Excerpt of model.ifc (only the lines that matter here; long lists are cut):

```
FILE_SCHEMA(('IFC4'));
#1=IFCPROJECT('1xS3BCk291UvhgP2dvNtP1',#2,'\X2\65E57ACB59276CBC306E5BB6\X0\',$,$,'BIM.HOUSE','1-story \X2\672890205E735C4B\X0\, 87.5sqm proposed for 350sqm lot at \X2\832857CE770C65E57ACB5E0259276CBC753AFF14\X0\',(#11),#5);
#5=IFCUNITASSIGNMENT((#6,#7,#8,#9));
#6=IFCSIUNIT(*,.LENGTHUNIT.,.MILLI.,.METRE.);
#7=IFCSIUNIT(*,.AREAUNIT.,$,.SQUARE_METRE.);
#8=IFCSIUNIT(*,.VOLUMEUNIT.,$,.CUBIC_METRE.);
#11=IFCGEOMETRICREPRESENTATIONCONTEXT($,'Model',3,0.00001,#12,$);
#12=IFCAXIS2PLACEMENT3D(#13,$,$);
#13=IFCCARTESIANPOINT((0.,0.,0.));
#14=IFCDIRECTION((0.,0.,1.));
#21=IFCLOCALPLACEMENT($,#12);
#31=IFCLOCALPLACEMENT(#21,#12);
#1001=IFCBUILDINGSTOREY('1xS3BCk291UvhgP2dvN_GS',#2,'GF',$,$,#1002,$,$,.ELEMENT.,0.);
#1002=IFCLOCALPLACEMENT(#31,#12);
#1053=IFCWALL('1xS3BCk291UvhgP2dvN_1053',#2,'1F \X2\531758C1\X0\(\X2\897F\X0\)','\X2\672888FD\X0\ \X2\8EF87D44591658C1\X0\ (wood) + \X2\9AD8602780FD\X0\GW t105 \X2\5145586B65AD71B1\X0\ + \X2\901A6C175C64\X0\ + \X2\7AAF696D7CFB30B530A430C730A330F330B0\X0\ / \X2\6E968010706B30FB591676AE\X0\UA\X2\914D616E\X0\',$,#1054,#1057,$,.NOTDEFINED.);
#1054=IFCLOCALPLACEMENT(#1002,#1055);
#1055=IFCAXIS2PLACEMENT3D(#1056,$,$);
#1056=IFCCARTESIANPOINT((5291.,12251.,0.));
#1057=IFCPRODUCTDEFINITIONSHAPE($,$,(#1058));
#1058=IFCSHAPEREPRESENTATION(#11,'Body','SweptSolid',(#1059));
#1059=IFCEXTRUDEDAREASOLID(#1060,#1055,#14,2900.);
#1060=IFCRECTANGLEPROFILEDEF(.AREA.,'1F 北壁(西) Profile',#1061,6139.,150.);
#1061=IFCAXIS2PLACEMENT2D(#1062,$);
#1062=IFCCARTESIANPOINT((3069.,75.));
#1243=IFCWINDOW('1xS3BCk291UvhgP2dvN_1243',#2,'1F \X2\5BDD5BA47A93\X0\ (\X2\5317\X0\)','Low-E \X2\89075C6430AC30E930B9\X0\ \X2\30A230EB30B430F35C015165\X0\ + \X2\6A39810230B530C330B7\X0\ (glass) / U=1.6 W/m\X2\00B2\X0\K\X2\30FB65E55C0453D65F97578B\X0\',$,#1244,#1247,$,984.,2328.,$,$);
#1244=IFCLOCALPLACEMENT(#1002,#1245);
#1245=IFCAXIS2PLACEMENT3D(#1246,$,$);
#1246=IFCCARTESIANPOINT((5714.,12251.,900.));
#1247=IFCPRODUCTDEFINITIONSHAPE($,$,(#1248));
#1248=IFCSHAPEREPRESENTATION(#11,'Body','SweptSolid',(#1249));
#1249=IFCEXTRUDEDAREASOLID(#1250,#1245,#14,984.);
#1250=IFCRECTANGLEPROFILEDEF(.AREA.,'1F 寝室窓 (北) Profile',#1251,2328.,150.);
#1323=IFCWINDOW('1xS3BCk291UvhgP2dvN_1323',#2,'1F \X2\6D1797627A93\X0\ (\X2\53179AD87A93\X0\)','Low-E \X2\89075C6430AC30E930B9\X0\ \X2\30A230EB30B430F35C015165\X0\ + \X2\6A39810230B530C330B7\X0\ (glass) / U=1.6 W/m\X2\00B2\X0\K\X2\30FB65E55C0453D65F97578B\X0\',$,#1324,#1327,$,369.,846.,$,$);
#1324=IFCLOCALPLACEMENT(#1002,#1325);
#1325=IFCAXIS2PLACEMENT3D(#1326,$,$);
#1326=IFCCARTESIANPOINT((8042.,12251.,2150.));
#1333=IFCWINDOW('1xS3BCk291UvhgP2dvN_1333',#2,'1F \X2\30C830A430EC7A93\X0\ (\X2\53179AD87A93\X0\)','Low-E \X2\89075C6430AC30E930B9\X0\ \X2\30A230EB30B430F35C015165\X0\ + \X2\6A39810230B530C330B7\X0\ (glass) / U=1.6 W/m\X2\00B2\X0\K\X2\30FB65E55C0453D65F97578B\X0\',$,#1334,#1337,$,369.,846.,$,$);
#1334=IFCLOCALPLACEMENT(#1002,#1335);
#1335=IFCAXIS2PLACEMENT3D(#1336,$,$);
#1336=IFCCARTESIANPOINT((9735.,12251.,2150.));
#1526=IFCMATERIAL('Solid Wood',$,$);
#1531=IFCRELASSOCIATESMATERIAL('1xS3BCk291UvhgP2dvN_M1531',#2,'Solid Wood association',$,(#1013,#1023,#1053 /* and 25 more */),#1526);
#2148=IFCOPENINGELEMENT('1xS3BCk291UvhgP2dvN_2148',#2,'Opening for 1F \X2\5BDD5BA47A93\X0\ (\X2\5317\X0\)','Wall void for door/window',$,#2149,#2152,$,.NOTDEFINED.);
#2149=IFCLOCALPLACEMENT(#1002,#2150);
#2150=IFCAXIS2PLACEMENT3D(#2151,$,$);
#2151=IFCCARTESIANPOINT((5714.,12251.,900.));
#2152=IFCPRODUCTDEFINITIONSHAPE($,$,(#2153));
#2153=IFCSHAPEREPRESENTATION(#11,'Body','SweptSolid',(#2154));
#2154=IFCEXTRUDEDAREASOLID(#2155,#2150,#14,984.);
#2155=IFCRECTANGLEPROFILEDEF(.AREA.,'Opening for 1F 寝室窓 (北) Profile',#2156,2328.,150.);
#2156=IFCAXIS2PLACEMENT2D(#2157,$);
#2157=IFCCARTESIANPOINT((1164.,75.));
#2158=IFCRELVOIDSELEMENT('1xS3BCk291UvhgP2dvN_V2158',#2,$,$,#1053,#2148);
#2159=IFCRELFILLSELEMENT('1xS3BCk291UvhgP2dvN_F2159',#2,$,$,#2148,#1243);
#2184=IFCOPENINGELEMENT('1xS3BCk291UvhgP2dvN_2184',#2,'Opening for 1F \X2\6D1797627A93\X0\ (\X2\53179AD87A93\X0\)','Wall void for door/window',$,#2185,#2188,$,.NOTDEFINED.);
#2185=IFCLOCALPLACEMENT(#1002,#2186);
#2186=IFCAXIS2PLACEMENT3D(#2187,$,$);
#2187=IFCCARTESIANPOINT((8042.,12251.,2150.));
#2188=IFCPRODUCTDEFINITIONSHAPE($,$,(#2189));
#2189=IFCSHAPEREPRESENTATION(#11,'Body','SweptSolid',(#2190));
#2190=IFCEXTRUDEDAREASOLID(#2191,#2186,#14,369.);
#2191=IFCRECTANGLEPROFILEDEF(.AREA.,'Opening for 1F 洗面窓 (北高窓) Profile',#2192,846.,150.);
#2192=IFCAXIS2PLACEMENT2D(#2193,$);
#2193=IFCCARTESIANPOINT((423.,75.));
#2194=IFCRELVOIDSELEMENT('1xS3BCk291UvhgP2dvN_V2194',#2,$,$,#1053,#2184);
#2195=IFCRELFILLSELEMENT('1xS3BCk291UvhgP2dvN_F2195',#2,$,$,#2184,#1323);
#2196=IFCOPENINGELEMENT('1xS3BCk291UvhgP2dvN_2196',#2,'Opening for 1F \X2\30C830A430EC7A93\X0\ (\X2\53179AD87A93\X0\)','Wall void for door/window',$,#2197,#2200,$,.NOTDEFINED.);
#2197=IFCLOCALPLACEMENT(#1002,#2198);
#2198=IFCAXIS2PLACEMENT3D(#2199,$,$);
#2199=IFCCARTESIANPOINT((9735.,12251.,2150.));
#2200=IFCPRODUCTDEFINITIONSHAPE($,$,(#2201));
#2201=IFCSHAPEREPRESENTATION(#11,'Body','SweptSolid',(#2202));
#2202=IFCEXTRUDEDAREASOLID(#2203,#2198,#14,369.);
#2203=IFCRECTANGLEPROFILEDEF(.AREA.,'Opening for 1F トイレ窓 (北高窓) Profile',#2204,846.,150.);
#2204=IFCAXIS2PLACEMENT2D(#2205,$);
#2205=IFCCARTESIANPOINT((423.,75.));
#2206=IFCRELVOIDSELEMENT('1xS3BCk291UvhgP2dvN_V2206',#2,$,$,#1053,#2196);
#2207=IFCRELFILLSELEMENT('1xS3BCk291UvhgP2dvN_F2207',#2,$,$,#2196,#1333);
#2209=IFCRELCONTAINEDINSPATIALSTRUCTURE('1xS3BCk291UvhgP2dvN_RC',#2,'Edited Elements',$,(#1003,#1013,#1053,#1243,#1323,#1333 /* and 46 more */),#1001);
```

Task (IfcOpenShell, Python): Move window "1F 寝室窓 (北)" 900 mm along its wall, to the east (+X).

```python
import ifcopenshell
import ifcopenshell.api.geometry
import ifcopenshell.util.placement
import ifcopenshell.util.unit

model = ifcopenshell.open("model.ifc")
unit_scale = ifcopenshell.util.unit.calculate_unit_scale(model)

window = model.by_guid("1xS3BCk291UvhgP2dvN_1243")
opening = window.FillsVoids[0].RelatingOpeningElement
wall = opening.VoidsElements[0].RelatingBuildingElement

wall_matrix = ifcopenshell.util.placement.get_local_placement(wall.ObjectPlacement)
shift = wall_matrix[:3, 0] * 0.9 / unit_scale
before = ifcopenshell.util.placement.get_local_placement(window.ObjectPlacement)[:3, 3].copy()

# The window is not placed relative to its opening, so move both.
for product in (opening, window):
    matrix = ifcopenshell.util.placement.get_local_placement(product.ObjectPlacement)
    matrix[:3, 3] += shift
    ifcopenshell.api.geometry.edit_object_placement(model, product=product, matrix=matrix, is_si=False)

after = ifcopenshell.util.placement.get_local_placement(window.ObjectPlacement)[:3, 3]
print("window moved by", (after - before).round(3) + 0.0)

model.write("model-out.ifc")
```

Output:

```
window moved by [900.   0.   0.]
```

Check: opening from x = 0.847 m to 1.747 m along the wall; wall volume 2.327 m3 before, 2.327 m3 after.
